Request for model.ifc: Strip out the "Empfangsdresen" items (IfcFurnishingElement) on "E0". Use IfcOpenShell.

First a look at what the model holds.

```python
import ifcopenshell
import ifcopenshell.util.element

model = ifcopenshell.open("model.ifc")
print(model.schema)
storey = next(s for s in model.by_type("IfcBuildingStorey") if s.Name == "E0")
furniture = [e for e in ifcopenshell.util.element.get_decomposition(storey) if e.is_a("IfcFurnishingElement")]
seen = {}
for e in furniture:
    element_type = ifcopenshell.util.element.get_type(e)
    name = element_type.Name if element_type not in (None, e) else None
    seen[name] = seen.get(name, 0) + 1
for name, count in sorted(seen.items(), key=str):
    print(count, "x", name)
```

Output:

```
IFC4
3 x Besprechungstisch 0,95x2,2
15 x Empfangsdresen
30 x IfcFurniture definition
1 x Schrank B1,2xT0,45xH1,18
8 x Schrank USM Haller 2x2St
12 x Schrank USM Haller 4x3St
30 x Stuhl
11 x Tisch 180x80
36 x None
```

```python
import ifcopenshell
import ifcopenshell.api.root
import ifcopenshell.util.element

model = ifcopenshell.open("model.ifc")

storey = next(s for s in model.by_type("IfcBuildingStorey") if s.Name == "E0")
furniture = [e for e in ifcopenshell.util.element.get_decomposition(storey) if e.is_a("IfcFurnishingElement")]
targets = [e for e in furniture if (t := ifcopenshell.util.element.get_type(e)) not in (None, e) and t.Name == "Empfangsdresen"]

for e in targets:
    ifcopenshell.api.root.remove_product(model, product=e)
print(len(targets), "removed")

model.write("model_rev.ifc")
```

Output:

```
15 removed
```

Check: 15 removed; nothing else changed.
